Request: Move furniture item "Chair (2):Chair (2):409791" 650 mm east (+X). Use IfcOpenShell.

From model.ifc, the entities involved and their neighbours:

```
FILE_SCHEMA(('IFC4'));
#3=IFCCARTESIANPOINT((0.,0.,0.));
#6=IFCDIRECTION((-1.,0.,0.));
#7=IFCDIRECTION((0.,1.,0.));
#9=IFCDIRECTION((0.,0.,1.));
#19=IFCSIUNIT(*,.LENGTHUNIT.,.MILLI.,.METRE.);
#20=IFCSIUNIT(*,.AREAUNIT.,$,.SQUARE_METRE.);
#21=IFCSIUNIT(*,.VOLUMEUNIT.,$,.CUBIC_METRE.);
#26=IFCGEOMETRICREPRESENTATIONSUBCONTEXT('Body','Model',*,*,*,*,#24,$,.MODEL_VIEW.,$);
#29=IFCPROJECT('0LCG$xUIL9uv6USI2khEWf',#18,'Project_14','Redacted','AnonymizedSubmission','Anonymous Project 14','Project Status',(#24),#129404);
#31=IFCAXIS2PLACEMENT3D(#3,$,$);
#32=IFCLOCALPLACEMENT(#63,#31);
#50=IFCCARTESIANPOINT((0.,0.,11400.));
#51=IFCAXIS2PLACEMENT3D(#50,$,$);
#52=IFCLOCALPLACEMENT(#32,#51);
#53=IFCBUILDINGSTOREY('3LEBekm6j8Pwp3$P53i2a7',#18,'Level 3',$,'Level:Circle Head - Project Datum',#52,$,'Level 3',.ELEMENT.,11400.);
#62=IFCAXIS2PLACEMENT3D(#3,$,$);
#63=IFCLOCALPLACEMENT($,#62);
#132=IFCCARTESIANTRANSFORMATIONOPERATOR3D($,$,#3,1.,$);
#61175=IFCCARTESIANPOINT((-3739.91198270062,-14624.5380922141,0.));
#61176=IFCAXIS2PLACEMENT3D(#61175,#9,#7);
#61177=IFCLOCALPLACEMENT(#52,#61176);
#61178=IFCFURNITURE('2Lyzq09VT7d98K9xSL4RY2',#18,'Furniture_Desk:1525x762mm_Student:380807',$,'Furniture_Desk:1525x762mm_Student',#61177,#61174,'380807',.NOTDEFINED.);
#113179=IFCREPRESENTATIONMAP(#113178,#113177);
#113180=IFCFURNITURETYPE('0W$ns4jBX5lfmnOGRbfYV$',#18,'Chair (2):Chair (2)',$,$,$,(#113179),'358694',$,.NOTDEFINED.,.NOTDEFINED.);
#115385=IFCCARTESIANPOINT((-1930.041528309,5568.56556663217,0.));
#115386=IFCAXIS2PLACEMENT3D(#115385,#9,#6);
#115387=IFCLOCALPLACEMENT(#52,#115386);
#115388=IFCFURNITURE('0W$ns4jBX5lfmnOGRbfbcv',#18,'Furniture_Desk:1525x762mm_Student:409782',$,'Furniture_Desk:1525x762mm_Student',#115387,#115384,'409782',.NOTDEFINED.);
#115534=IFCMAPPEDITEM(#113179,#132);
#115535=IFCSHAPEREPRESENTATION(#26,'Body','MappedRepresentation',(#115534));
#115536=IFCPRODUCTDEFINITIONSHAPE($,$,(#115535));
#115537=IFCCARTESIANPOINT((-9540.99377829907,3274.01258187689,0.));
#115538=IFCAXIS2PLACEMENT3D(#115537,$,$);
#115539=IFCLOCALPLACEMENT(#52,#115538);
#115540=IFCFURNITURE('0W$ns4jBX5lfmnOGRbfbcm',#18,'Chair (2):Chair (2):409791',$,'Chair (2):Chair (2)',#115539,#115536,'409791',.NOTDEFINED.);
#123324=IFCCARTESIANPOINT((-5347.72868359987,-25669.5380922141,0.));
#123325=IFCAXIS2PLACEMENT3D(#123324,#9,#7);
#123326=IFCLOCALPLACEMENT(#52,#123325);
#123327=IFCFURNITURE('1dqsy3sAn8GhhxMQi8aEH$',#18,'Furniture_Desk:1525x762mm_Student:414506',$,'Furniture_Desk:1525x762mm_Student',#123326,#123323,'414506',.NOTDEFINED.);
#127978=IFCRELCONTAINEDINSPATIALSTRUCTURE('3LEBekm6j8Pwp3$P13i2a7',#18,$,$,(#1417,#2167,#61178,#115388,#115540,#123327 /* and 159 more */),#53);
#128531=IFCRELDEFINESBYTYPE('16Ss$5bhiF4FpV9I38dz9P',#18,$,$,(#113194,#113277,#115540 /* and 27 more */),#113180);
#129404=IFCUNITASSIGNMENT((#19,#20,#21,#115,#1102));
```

```python
import ifcopenshell
import ifcopenshell.api.geometry
import ifcopenshell.util.placement
import ifcopenshell.util.unit

model = ifcopenshell.open("model.ifc")
unit_scale = ifcopenshell.util.unit.calculate_unit_scale(model)

item = model.by_guid("0W$ns4jBX5lfmnOGRbfbcm")
matrix = ifcopenshell.util.placement.get_local_placement(item.ObjectPlacement)
matrix[0, 3] += 0.65 / unit_scale
ifcopenshell.api.geometry.edit_object_placement(model, product=item, matrix=matrix, is_si=False)

print(ifcopenshell.util.placement.get_local_placement(item.ObjectPlacement).round(3) + 0.0)

model.write("model-out.ifc")
```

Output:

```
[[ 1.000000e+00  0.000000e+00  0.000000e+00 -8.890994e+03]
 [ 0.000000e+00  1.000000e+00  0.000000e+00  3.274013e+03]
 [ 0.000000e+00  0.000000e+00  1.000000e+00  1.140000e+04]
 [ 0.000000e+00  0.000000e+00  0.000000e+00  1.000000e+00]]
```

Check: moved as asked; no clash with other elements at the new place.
